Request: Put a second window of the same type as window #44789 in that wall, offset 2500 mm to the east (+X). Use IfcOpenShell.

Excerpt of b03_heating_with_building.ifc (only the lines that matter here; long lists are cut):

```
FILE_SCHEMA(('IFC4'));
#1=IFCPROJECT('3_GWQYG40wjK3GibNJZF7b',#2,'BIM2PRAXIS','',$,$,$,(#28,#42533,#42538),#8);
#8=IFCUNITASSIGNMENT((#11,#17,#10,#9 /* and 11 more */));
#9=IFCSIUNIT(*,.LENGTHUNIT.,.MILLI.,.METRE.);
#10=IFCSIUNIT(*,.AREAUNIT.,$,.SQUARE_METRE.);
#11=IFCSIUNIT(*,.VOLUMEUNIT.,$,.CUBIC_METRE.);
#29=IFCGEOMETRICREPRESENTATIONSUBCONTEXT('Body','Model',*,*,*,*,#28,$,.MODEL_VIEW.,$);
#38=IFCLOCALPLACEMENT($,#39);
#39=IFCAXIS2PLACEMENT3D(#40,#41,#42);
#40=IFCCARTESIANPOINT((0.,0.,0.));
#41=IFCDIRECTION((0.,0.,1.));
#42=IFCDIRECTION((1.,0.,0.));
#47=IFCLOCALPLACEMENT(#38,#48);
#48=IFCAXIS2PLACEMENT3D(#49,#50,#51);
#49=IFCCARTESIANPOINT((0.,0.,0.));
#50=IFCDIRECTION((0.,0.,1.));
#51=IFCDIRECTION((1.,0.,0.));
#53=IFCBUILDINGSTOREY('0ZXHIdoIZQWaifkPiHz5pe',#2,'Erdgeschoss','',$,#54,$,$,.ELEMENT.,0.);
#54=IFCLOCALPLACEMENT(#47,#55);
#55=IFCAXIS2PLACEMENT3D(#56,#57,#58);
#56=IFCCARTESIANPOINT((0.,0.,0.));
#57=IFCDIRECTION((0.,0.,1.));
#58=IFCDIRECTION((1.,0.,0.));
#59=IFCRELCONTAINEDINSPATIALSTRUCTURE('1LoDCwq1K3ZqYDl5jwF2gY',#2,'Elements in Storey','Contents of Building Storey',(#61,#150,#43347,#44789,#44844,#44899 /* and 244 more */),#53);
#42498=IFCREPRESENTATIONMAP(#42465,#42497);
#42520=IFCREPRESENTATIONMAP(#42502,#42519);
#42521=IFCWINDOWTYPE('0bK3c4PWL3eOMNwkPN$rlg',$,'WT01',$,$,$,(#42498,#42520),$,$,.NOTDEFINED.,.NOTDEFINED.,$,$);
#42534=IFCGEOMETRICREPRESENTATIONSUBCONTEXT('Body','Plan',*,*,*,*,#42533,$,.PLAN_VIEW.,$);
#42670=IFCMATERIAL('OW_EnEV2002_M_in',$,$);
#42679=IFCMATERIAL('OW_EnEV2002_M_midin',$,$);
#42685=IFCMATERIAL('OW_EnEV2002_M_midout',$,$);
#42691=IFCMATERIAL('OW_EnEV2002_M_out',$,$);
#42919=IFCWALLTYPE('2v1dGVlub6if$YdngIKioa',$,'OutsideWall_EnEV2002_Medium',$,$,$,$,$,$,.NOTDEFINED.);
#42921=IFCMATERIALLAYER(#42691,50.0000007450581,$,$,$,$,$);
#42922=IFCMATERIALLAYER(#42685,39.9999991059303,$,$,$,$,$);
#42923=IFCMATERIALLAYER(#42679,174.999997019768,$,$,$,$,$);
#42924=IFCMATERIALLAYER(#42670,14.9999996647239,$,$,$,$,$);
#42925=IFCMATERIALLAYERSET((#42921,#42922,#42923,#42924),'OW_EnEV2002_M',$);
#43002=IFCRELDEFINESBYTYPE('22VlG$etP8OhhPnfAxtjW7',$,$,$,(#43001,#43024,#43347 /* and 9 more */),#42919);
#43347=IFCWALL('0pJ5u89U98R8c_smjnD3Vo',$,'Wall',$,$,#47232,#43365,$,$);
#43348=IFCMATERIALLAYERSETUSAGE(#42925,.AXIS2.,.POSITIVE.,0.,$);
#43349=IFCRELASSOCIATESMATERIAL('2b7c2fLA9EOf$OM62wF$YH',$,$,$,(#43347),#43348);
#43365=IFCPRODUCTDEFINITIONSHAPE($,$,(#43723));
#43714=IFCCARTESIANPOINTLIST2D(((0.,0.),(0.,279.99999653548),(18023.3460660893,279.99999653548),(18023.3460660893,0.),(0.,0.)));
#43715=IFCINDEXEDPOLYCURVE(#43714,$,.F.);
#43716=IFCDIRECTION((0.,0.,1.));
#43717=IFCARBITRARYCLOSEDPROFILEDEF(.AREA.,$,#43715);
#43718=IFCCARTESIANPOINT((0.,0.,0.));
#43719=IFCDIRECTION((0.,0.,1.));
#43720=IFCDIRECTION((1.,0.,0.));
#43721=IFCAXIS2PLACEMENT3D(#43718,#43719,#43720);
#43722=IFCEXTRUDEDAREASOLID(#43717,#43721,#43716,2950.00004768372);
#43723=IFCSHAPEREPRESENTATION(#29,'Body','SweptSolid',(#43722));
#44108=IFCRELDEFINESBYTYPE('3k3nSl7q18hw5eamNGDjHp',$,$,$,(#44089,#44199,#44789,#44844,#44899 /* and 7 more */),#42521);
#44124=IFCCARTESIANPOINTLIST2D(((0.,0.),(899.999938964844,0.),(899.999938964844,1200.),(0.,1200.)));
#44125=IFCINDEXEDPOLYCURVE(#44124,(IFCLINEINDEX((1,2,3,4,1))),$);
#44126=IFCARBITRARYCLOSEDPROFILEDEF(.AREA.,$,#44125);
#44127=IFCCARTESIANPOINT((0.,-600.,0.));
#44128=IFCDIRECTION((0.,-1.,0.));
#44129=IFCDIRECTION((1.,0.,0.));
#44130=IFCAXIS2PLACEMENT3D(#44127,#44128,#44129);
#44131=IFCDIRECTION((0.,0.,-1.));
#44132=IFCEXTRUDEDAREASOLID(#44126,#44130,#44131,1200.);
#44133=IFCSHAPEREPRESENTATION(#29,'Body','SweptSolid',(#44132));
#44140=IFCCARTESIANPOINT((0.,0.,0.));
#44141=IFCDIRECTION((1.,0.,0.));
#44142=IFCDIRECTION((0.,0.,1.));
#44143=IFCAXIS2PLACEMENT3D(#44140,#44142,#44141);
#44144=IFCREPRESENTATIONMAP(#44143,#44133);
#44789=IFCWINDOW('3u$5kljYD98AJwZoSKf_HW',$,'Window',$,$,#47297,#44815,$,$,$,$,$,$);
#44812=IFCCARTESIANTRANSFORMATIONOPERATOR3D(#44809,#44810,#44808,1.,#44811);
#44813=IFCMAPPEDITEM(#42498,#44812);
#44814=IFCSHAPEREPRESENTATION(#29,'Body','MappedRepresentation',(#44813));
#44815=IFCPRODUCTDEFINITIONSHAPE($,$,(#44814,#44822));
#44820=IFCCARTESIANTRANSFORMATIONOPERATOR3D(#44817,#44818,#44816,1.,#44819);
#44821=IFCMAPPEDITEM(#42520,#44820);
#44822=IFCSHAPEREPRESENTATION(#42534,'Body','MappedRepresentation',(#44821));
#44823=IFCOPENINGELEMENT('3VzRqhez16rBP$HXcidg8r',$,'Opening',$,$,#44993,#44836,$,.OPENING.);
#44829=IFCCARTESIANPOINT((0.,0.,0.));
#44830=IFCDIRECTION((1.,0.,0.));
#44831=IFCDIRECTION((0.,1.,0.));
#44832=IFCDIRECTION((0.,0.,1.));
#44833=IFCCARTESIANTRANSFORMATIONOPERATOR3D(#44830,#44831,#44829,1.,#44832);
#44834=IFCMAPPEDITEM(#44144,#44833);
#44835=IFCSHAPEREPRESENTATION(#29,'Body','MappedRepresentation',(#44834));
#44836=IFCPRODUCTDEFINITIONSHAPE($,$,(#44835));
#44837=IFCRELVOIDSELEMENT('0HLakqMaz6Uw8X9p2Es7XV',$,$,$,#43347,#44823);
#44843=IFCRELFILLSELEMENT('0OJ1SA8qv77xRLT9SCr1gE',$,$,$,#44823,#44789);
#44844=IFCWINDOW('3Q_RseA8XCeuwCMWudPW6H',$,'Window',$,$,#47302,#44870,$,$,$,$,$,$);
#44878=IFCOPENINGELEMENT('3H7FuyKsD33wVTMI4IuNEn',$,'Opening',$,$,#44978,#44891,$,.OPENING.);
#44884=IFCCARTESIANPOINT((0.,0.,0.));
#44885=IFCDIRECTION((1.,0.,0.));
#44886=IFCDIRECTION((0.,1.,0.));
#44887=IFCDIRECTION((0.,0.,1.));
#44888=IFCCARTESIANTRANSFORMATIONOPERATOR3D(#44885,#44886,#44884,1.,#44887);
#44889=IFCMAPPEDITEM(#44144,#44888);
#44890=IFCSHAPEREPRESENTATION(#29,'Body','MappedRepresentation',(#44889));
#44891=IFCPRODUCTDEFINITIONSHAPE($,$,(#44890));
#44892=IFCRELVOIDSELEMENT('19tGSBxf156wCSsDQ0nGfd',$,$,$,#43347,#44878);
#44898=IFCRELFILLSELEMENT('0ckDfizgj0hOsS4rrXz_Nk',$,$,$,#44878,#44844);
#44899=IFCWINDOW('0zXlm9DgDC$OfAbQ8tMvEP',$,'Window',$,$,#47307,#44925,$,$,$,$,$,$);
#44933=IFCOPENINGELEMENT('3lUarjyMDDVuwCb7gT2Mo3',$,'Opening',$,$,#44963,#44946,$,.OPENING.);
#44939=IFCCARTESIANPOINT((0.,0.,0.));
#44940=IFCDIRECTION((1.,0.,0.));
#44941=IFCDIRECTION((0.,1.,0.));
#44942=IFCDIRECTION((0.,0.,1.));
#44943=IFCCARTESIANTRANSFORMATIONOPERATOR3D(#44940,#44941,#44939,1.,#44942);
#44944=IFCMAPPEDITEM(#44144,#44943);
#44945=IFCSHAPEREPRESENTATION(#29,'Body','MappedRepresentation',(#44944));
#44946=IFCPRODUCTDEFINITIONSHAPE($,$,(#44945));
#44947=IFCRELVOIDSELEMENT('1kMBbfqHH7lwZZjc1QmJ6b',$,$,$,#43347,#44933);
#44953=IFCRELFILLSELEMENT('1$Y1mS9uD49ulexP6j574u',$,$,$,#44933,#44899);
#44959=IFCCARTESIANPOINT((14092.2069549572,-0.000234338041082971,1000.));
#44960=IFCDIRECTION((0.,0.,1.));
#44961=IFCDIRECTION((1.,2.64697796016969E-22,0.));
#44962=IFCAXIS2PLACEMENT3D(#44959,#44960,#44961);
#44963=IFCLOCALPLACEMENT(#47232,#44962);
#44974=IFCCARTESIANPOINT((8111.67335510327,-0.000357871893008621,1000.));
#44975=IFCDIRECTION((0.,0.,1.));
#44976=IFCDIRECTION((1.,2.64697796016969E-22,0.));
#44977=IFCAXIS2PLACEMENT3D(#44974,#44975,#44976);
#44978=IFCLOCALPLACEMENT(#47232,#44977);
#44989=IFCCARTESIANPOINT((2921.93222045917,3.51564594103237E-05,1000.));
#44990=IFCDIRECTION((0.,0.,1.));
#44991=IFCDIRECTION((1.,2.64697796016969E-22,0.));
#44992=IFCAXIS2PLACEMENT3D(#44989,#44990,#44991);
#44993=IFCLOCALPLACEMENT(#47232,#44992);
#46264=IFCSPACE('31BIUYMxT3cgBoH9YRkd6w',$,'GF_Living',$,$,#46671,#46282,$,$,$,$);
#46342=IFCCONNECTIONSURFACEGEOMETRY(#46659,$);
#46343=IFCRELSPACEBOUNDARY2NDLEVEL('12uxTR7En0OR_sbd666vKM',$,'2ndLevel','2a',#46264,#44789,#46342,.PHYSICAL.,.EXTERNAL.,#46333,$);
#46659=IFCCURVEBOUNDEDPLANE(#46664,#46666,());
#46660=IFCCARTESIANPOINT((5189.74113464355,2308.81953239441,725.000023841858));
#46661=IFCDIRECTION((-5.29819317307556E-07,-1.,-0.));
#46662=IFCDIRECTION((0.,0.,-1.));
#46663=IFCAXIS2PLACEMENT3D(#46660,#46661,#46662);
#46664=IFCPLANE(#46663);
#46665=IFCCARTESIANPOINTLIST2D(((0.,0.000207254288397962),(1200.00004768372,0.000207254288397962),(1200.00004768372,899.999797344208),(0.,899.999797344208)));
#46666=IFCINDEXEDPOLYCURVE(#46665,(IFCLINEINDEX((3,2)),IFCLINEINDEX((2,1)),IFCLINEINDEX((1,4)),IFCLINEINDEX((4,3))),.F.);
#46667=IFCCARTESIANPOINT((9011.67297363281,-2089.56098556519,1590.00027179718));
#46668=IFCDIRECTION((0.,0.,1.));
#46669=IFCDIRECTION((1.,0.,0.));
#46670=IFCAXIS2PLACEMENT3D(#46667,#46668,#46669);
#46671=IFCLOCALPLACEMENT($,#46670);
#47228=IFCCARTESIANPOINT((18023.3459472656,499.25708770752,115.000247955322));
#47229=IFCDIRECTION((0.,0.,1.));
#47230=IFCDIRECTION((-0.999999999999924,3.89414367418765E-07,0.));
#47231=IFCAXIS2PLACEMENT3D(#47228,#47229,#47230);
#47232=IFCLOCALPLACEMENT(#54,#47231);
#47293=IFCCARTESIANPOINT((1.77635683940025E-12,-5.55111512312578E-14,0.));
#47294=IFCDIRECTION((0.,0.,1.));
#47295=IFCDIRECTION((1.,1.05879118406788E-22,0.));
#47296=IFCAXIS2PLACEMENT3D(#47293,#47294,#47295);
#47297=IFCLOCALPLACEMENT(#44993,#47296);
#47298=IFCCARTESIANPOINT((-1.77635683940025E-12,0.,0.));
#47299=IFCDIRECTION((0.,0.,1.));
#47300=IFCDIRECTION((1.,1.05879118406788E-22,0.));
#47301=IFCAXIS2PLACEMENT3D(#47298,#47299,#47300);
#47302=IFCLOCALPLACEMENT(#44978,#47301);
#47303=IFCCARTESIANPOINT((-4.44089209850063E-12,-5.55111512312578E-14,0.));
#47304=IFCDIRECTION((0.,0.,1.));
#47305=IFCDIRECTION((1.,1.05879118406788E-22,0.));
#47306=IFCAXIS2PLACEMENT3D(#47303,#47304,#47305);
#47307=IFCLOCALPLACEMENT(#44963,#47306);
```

```python
import numpy as np
import ifcopenshell
import ifcopenshell.api.feature
import ifcopenshell.api.geometry
import ifcopenshell.api.root
import ifcopenshell.geom
import ifcopenshell.util.element
import ifcopenshell.util.placement
import ifcopenshell.util.shape
import ifcopenshell.util.unit

model = ifcopenshell.open("b03_heating_with_building.ifc")
unit_scale = ifcopenshell.util.unit.calculate_unit_scale(model)
settings = ifcopenshell.geom.settings()


def volume(element):
    """Net volume in cubic metres, openings subtracted."""
    shape = ifcopenshell.geom.create_shape(settings, element)
    return ifcopenshell.util.shape.get_volume(shape.geometry)


window = model.by_guid("3u$5kljYD98AJwZoSKf_HW")
opening = window.FillsVoids[0].RelatingOpeningElement
wall = opening.VoidsElements[0].RelatingBuildingElement
before = volume(wall)
shift = ifcopenshell.util.placement.get_local_placement(wall.ObjectPlacement)[:3, 0] * -2.5 / unit_scale

# copy_class copies the void relationship, type, container and properties, but no geometry.
new_opening = ifcopenshell.api.root.copy_class(model, product=opening)
new_opening.Representation = ifcopenshell.util.element.copy_deep(
    model, opening.Representation, exclude=["IfcGeometricRepresentationContext", "IfcRepresentationMap"]
)
new_window = ifcopenshell.api.root.copy_class(model, product=window)
new_window.Representation = ifcopenshell.util.element.copy_deep(
    model, window.Representation, exclude=["IfcGeometricRepresentationContext", "IfcRepresentationMap"]
)
ifcopenshell.api.feature.add_filling(model, opening=new_opening, element=new_window)

for old, new in ((opening, new_opening), (window, new_window)):
    matrix = ifcopenshell.util.placement.get_local_placement(old.ObjectPlacement)
    matrix[:3, 3] += shift
    ifcopenshell.api.geometry.edit_object_placement(model, product=new, matrix=matrix, is_si=False)

# The copied space boundaries still share their surfaces with the original.
for rel in new_window.ProvidesBoundaries:
    if rel.ConnectionGeometry:
        rel.ConnectionGeometry = ifcopenshell.util.element.copy_deep(model, rel.ConnectionGeometry)

# Space boundary surfaces are stored in each space's coordinates; move them too.
for rel in new_window.ProvidesBoundaries:
    if not rel.ConnectionGeometry:
        continue
    surface = rel.ConnectionGeometry.SurfaceOnRelatingElement.BasisSurface
    space_matrix = ifcopenshell.util.placement.get_local_placement(rel.RelatingSpace.ObjectPlacement)
    point = np.array(surface.Position.Location.Coordinates) + space_matrix[:3, :3].T @ shift
    surface.Position = model.createIfcAxis2Placement3D(
        model.createIfcCartesianPoint(point.tolist()), surface.Position.Axis, surface.Position.RefDirection
    )

after = volume(wall)

print(f"wall volume {before:.3f} -> {after:.3f} m3")

model.write("b03_heating_with_building-out.ifc")
```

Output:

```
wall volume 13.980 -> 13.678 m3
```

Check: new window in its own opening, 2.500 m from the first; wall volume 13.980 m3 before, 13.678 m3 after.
